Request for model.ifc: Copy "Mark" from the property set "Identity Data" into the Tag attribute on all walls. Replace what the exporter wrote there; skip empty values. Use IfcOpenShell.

First a look at what the model holds.

```python
import ifcopenshell
import ifcopenshell.util.element

model = ifcopenshell.open("model.ifc")
print(model.schema)
walls = model.by_type("IfcWall")
print(len(walls), "walls")
for e in walls[:8]:
    source = ifcopenshell.util.element.get_pset(e, "Identity Data", "Mark")
    target = e.Tag
    print(e.id(), repr(source), repr(target), sep=" | ")
```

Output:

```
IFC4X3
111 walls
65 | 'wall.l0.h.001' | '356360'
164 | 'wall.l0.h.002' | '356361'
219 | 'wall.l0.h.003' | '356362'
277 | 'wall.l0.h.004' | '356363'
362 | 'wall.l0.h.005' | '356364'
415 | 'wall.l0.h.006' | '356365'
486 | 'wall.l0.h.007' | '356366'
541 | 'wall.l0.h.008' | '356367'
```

```python
import ifcopenshell
import ifcopenshell.util.element

model = ifcopenshell.open("model.ifc")

count = 0
for e in model.by_type("IfcWall"):
    value = ifcopenshell.util.element.get_pset(e, "Identity Data", "Mark")
    current = e.Tag
    if not value or not value.strip() or current == value:
        continue
    e.Tag = value
    count += 1

print(count, "walls updated")

model.write("model_updated.ifc")
```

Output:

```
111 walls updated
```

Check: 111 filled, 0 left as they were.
